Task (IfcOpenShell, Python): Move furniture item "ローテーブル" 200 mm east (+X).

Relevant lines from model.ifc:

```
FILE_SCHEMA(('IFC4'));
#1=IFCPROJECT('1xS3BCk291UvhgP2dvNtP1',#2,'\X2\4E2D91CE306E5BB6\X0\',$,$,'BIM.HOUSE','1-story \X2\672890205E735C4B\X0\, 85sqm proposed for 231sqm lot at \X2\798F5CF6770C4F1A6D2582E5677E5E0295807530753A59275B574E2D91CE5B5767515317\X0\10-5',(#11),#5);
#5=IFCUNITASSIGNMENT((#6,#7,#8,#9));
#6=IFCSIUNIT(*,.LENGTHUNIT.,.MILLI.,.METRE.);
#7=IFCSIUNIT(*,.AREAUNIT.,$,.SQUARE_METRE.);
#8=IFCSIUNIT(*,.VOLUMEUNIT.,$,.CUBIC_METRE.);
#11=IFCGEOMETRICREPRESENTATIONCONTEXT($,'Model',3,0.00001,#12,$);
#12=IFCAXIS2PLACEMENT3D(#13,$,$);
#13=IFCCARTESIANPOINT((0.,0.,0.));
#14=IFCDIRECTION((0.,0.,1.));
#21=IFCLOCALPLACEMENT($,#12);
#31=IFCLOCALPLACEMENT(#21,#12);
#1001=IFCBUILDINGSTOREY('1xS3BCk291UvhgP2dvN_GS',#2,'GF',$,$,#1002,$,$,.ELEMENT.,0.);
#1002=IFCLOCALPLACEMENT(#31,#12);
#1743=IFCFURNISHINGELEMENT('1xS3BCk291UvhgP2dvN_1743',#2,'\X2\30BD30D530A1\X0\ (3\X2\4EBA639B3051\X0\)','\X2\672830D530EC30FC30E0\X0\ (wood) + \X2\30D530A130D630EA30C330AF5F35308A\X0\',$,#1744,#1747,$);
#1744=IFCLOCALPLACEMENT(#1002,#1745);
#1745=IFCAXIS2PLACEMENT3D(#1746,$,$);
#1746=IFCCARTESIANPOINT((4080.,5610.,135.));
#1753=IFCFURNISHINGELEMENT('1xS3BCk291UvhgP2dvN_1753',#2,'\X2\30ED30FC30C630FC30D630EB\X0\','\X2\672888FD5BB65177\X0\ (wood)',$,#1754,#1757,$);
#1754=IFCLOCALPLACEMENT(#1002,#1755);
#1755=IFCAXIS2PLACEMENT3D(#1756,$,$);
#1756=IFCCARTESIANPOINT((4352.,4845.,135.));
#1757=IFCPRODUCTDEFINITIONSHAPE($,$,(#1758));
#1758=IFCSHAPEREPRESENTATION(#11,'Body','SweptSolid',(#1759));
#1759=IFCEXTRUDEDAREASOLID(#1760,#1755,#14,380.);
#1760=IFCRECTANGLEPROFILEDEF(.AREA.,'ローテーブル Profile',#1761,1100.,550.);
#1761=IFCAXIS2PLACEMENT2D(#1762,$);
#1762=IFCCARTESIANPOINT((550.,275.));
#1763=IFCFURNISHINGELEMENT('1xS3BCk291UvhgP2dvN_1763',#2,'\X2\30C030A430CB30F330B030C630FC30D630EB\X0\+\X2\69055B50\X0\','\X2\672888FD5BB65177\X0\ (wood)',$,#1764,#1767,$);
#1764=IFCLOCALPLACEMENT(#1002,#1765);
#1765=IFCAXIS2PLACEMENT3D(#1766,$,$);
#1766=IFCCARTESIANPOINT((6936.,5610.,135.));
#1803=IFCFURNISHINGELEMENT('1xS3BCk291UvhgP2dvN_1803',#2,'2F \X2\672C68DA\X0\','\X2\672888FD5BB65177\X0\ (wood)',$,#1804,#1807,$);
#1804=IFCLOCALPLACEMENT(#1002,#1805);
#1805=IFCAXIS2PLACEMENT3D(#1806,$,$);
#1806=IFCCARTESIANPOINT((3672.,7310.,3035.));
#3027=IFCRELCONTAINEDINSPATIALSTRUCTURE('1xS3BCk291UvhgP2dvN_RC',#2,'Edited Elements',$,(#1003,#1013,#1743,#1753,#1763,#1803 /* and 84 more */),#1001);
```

```python
import ifcopenshell
import ifcopenshell.api.geometry
import ifcopenshell.util.placement
import ifcopenshell.util.unit

model = ifcopenshell.open("model.ifc")
unit_scale = ifcopenshell.util.unit.calculate_unit_scale(model)

item = model.by_id(1753)
matrix = ifcopenshell.util.placement.get_local_placement(item.ObjectPlacement)
matrix[0, 3] += 0.2 / unit_scale
ifcopenshell.api.geometry.edit_object_placement(model, product=item, matrix=matrix, is_si=False)

print(ifcopenshell.util.placement.get_local_placement(item.ObjectPlacement).round(3) + 0.0)

model.write("model_edited.ifc")
```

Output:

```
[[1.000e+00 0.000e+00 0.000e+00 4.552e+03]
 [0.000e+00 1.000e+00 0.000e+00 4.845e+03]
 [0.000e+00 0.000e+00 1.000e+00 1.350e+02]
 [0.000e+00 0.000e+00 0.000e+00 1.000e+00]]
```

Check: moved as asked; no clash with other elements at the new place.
